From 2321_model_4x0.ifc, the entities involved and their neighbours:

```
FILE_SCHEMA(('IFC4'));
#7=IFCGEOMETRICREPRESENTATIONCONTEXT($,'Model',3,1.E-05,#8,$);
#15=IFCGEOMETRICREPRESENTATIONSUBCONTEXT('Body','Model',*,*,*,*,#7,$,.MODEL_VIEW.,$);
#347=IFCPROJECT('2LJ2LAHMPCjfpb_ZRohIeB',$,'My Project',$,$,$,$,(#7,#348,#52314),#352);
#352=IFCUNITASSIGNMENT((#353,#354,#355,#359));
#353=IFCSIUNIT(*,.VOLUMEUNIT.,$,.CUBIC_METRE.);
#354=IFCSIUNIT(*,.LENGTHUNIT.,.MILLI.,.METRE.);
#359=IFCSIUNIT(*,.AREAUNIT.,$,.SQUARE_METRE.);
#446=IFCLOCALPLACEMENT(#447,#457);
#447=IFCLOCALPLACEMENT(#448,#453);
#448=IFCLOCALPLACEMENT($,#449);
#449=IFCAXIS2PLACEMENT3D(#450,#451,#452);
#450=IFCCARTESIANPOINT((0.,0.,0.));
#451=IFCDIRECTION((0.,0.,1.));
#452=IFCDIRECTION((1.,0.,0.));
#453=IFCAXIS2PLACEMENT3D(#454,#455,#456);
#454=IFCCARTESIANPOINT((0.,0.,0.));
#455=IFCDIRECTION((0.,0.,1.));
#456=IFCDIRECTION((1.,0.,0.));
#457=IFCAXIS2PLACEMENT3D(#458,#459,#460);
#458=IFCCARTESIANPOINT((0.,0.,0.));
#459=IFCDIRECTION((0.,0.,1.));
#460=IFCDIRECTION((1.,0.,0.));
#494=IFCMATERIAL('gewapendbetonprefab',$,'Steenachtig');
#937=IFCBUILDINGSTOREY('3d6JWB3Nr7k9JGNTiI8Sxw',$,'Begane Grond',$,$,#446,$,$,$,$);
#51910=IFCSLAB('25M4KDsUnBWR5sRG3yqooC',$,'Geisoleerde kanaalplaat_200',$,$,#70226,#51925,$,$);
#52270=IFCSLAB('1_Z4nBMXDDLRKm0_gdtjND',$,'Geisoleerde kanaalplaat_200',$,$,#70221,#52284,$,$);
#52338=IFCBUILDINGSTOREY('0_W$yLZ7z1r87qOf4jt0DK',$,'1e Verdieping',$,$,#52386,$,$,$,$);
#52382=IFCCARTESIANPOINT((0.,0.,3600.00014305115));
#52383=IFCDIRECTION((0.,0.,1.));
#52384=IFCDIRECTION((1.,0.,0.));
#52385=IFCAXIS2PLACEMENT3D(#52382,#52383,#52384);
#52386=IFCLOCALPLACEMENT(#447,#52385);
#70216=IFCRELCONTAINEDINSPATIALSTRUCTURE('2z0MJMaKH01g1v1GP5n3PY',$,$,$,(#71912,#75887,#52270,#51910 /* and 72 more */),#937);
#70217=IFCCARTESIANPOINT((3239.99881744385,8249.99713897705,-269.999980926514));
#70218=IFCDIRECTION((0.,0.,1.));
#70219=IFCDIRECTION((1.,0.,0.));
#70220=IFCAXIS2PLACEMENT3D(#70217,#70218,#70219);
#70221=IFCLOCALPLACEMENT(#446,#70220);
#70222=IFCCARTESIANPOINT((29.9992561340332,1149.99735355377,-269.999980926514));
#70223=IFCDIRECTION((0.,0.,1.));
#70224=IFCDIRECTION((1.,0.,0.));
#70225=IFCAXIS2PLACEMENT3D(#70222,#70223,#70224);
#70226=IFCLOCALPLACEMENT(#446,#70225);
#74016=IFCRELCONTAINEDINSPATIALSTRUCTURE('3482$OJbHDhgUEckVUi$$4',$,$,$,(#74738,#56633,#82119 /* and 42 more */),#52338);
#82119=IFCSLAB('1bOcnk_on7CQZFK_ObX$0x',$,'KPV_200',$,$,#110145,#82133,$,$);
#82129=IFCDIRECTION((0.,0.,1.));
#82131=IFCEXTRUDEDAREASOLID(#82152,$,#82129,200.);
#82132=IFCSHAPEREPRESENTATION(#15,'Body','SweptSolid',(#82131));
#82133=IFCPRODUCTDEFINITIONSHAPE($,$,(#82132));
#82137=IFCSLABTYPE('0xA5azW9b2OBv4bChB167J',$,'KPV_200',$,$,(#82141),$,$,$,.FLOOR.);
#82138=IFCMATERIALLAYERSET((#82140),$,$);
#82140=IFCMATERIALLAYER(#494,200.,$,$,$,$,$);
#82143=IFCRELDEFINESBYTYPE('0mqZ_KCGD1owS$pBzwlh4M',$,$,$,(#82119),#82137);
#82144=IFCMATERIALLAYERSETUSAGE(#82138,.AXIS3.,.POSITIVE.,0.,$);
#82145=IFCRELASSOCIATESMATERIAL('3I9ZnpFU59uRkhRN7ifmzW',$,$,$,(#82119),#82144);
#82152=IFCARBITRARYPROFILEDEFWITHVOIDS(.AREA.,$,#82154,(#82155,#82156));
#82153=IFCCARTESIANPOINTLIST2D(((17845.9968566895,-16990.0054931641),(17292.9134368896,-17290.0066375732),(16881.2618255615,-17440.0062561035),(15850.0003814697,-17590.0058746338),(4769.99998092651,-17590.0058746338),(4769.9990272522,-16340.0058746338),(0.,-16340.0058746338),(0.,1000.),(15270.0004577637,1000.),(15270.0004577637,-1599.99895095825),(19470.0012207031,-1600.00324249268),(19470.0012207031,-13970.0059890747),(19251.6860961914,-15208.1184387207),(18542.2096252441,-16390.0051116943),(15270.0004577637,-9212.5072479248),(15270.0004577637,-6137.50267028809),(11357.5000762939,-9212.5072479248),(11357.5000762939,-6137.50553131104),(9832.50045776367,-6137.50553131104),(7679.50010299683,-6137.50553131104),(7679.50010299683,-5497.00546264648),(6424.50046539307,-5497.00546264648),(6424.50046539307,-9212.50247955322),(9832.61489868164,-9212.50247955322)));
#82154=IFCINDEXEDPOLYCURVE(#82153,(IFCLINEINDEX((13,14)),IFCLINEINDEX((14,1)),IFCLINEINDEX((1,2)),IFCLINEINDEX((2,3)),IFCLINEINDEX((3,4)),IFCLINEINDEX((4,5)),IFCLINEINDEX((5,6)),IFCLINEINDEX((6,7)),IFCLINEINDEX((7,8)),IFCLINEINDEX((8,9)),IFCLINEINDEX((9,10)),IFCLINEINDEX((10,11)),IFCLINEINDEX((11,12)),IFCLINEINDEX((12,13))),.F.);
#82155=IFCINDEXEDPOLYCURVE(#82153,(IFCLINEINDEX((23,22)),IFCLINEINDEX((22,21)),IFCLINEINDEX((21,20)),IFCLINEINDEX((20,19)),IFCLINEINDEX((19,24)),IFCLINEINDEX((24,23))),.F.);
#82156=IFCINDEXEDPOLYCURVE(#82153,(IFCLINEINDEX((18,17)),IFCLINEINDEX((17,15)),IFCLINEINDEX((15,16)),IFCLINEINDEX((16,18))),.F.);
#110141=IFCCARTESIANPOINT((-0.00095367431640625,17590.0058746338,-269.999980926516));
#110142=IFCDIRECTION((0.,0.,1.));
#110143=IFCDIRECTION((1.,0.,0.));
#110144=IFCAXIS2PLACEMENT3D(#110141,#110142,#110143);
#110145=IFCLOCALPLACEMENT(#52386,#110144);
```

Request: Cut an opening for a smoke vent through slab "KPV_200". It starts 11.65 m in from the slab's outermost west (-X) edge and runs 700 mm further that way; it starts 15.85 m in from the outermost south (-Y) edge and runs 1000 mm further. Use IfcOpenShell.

```python
import numpy as np
import ifcopenshell
import ifcopenshell.api.feature
import ifcopenshell.api.geometry
import ifcopenshell.api.root
import ifcopenshell.geom
import ifcopenshell.util.placement
import ifcopenshell.util.representation
import ifcopenshell.util.shape
import ifcopenshell.util.unit

model = ifcopenshell.open("2321_model_4x0.ifc")
unit_scale = ifcopenshell.util.unit.calculate_unit_scale(model)
settings = ifcopenshell.geom.settings()


def volume(element):
    """Net volume in cubic metres, openings subtracted."""
    shape = ifcopenshell.geom.create_shape(settings, element)
    return ifcopenshell.util.shape.get_volume(shape.geometry)


slab = model.by_guid("1bOcnk_on7CQZFK_ObX$0x")
before = volume(slab)

# Extent in the slab's own axes, in metres. The edges named are its -X and -Y sides.
slab_shape = ifcopenshell.geom.create_shape(settings, slab)
vertices = ifcopenshell.util.shape.get_vertices(slab_shape.geometry)
x_min, y_min, bottom = vertices.min(axis=0)
top = vertices[:, 2].max()

opening = ifcopenshell.api.root.create_entity(model, ifc_class="IfcOpeningElement", name="Smoke vent opening", predefined_type="OPENING")
context = ifcopenshell.util.representation.get_context(model, "Model", "Body", "MODEL_VIEW")
width, depth = 0.7, 1
outline = [(0.0, 0.0), (width, 0.0), (width, depth), (0.0, depth), (0.0, 0.0)]
# Overshoot both faces by 50 mm so the cut is clean.
shape = ifcopenshell.api.geometry.add_slab_representation(
    model, context=context, depth=top - bottom + 0.1, polyline=outline
)
ifcopenshell.api.geometry.assign_representation(model, product=opening, representation=shape)

matrix = ifcopenshell.util.placement.get_local_placement(slab.ObjectPlacement)
matrix[:, 3] = matrix @ np.append(np.array([x_min + 11.65, y_min + 15.85, bottom - 0.05]) / unit_scale, 1.0)
ifcopenshell.api.geometry.edit_object_placement(model, product=opening, matrix=matrix, is_si=False)
ifcopenshell.api.feature.add_feature(model, feature=opening, element=slab)

after = volume(slab)

print(f"slab volume {before:.3f} -> {after:.3f} m3")

model.write("2321_model_4x0-out.ifc")
```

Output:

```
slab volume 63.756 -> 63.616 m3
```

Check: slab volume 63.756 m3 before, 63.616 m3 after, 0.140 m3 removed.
